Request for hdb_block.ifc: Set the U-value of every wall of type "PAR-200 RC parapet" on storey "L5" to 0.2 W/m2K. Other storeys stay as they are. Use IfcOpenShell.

First a look at what the model holds.

```python
import ifcopenshell
import ifcopenshell.util.element

model = ifcopenshell.open("hdb_block.ifc")
print(model.schema)
storey = next(s for s in model.by_type("IfcBuildingStorey") if s.Name == "L5")
walls = [e for e in ifcopenshell.util.element.get_decomposition(storey) if e.is_a("IfcWall")]
seen = {}
for e in walls:
    element_type = ifcopenshell.util.element.get_type(e)
    key = (element_type.Name if element_type != e and element_type else None, ifcopenshell.util.element.get_pset(e, "Pset_WallCommon", "ThermalTransmittance"))
    seen[key] = seen.get(key, 0) + 1
for (name, value), count in sorted(seen.items(), key=str):
    print(count, "x", name, "|", value)
```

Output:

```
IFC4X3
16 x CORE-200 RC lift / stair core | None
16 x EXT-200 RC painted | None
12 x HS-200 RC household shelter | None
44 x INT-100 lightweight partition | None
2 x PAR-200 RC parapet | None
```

```python
import ifcopenshell
import ifcopenshell.api.pset
import ifcopenshell.util.element

model = ifcopenshell.open("hdb_block.ifc")

storey = next(s for s in model.by_type("IfcBuildingStorey") if s.Name == "L5")
walls = [e for e in ifcopenshell.util.element.get_decomposition(storey) if e.is_a("IfcWall")]

count = 0
for e in walls:
    element_type = ifcopenshell.util.element.get_type(e)
    if element_type in (None, e) or element_type.Name != "PAR-200 RC parapet":
        continue
    # add_pset returns the element's existing set when there is one.
    pset = ifcopenshell.api.pset.add_pset(model, product=e, name="Pset_WallCommon")
    ifcopenshell.api.pset.edit_pset(model, pset=pset, properties={"ThermalTransmittance": 0.2})
    count += 1

print(count, "walls updated")

model.write("hdb_block_edited.ifc")
```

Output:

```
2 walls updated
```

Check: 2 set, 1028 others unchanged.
